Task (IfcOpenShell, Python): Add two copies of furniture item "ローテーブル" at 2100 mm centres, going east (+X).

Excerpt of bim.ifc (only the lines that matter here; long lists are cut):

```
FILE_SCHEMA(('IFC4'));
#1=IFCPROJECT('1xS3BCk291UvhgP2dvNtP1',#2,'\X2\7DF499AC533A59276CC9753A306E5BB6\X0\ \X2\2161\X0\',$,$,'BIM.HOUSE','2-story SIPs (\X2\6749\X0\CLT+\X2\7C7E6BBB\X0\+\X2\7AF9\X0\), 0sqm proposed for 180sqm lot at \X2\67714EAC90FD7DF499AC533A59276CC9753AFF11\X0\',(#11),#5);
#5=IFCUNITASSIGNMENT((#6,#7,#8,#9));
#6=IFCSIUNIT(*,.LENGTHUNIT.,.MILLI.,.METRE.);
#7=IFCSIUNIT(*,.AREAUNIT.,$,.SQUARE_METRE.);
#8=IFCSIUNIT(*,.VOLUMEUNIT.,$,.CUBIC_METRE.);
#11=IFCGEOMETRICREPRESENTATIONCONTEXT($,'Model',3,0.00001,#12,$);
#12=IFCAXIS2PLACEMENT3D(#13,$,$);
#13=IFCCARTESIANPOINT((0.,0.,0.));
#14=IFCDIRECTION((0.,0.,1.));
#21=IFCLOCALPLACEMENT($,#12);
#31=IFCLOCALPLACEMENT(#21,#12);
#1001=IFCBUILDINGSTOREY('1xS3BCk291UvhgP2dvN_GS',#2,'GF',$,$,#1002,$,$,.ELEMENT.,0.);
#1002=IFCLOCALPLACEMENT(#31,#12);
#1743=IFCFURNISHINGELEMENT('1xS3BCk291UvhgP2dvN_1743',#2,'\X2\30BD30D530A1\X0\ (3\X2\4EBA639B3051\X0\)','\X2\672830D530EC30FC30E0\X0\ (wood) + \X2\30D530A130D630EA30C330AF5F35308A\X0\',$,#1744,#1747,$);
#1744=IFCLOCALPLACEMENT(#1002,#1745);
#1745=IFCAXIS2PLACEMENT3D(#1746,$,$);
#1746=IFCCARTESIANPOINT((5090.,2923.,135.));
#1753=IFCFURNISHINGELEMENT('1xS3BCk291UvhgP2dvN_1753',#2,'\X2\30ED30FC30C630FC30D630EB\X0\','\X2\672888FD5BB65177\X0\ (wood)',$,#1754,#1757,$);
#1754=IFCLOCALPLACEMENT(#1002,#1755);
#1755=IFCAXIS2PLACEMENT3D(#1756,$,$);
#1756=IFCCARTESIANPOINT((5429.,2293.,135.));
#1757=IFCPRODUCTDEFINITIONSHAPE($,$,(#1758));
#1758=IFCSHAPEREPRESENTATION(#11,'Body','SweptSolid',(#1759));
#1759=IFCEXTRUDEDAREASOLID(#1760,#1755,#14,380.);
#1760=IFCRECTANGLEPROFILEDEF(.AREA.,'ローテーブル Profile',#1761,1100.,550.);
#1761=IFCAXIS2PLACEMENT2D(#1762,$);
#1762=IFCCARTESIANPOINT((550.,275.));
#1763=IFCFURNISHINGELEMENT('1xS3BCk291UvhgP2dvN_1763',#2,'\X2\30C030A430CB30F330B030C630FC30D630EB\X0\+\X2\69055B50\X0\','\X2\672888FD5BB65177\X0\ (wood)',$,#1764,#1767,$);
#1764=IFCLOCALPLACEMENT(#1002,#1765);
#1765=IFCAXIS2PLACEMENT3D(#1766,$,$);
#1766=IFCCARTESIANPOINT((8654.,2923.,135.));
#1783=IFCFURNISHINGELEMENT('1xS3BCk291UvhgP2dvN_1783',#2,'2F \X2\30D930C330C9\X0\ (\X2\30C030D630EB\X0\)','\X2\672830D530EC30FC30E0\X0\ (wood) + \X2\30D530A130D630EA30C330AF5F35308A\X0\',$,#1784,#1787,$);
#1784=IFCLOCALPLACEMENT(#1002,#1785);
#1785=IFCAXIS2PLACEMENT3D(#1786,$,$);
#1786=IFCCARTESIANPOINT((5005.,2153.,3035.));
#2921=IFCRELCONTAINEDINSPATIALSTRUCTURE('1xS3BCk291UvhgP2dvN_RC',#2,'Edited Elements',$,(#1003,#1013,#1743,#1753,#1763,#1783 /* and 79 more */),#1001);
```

```python
import numpy as np
import ifcopenshell
import ifcopenshell.api.geometry
import ifcopenshell.api.root
import ifcopenshell.util.element
import ifcopenshell.util.placement
import ifcopenshell.util.unit

model = ifcopenshell.open("bim.ifc")
unit_scale = ifcopenshell.util.unit.calculate_unit_scale(model)


def reuse_history(source, copy):
    """copy_class also copies each property set's owner history, people and application; keep the originals."""
    for rel in copy.IsDefinedBy:
        if rel.is_a("IfcRelDefinesByProperties") and (history := rel.RelatingPropertyDefinition.OwnerHistory):
            rel.RelatingPropertyDefinition.OwnerHistory = source.OwnerHistory
            ifcopenshell.util.element.remove_deep2(model, history)


source = model.by_guid("1xS3BCk291UvhgP2dvN_1753")
base = ifcopenshell.util.placement.get_local_placement(source.ObjectPlacement)
step = np.array([1.0, 0.0, 0.0]) * 2.1 / unit_scale

for i in range(1, 3):
    copy = ifcopenshell.api.root.copy_class(model, product=source)
    copy.Representation = ifcopenshell.util.element.copy_deep(
        model, source.Representation, exclude=["IfcGeometricRepresentationContext", "IfcRepresentationMap"]
    )
    reuse_history(source, copy)
    matrix = base.copy()
    matrix[:3, 3] += i * step
    print("added at", matrix[:3, 3].round(3) + 0.0)
    ifcopenshell.api.geometry.edit_object_placement(model, product=copy, matrix=matrix, is_si=False)

model.write("bim_v2.ifc")
```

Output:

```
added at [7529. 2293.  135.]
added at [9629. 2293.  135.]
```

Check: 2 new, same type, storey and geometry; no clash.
